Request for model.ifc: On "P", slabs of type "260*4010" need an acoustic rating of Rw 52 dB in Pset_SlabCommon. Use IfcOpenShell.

First a look at what the model holds.

```python
import ifcopenshell
import ifcopenshell.util.element

model = ifcopenshell.open("model.ifc")
print(model.schema)
storey = next(s for s in model.by_type("IfcBuildingStorey") if s.Name == "P")
slabs = [e for e in ifcopenshell.util.element.get_decomposition(storey) if e.is_a("IfcSlab")]
seen = {}
for e in slabs:
    element_type = ifcopenshell.util.element.get_type(e)
    key = (element_type.Name if element_type != e and element_type else None, ifcopenshell.util.element.get_pset(e, "Pset_SlabCommon", "AcousticRating"))
    seen[key] = seen.get(key, 0) + 1
for (name, value), count in sorted(seen.items(), key=str):
    print(count, "x", name, "|", value)
```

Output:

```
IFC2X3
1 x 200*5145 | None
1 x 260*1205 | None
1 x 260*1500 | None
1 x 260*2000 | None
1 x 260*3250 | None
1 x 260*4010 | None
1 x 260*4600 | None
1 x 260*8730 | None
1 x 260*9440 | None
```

```python
import ifcopenshell
import ifcopenshell.api.pset
import ifcopenshell.util.element

model = ifcopenshell.open("model.ifc")

storey = next(s for s in model.by_type("IfcBuildingStorey") if s.Name == "P")
slabs = [e for e in ifcopenshell.util.element.get_decomposition(storey) if e.is_a("IfcSlab")]

count = 0
for e in slabs:
    element_type = ifcopenshell.util.element.get_type(e)
    if element_type in (None, e) or element_type.Name != "260*4010":
        continue
    found = ifcopenshell.util.element.get_pset(e, "Pset_SlabCommon", should_inherit=False)
    if found:
        pset = model.by_id(found["id"])
        if len(ifcopenshell.util.element.get_elements_by_pset(pset)) > 1:
            pset = ifcopenshell.api.pset.unshare_pset(model, products=[e], pset=pset)[0]
    else:
        pset = ifcopenshell.api.pset.add_pset(model, product=e, name="Pset_SlabCommon")
    ifcopenshell.api.pset.edit_pset(model, pset=pset, properties={"AcousticRating": "Rw 52 dB"})
    count += 1

print(count, "slabs updated")

model.write("model_edited.ifc")
```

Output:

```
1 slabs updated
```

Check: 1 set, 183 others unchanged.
